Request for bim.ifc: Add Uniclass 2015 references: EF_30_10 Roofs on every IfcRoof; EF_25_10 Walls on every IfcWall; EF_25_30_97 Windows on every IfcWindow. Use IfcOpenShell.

First a look at what the model holds.

```python
import ifcopenshell

model = ifcopenshell.open("bim.ifc")
print(model.schema)
print("classifications:", [c.Name for c in model.by_type("IfcClassification")])
for ifc_class in ("IfcDoor", "IfcRoof", "IfcStair", "IfcWall", "IfcWindow"):
    print(ifc_class, len(model.by_type(ifc_class)))
```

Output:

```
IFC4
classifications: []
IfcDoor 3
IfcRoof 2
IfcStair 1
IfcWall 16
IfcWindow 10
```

```python
import ifcopenshell
import ifcopenshell.api.classification

model = ifcopenshell.open("bim.ifc")

system = ifcopenshell.api.classification.add_classification(model, classification="Uniclass 2015")

codes = {
    "IfcRoof": ("EF_30_10", "Roofs"),
    "IfcWall": ("EF_25_10", "Walls"),
    "IfcWindow": ("EF_25_30_97", "Windows"),
}
for ifc_class, (code, name) in codes.items():
    products = model.by_type(ifc_class)
    ifcopenshell.api.classification.add_reference(
        model, products=products, classification=system, identification=code, name=name
    )
    print(code, len(products))

model.write("bim-out.ifc")
```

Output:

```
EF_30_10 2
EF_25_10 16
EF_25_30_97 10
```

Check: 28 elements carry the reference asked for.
